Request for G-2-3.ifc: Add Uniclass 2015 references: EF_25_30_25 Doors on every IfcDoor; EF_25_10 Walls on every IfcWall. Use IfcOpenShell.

First a look at what the model holds.

```python
import ifcopenshell

model = ifcopenshell.open("G-2-3.ifc")
print(model.schema)
print("classifications:", [c.Name for c in model.by_type("IfcClassification")])
for ifc_class in ("IfcDoor", "IfcRoof", "IfcStair", "IfcWall", "IfcWindow"):
    print(ifc_class, len(model.by_type(ifc_class)))
```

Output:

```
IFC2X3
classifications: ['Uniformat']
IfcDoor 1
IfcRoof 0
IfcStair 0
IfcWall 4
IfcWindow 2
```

```python
import ifcopenshell
import ifcopenshell.api.classification

model = ifcopenshell.open("G-2-3.ifc")

# IFC2X3 requires Source and Edition and has no link from the project to the system.
system = model.create_entity("IfcClassification", Source="NBS", Edition="2015", Name="Uniclass 2015")

codes = {
    "IfcDoor": ("EF_25_30_25", "Doors"),
    "IfcWall": ("EF_25_10", "Walls"),
}
for ifc_class, (code, name) in codes.items():
    products = model.by_type(ifc_class)
    ifcopenshell.api.classification.add_reference(
        model, products=products, classification=system, identification=code, name=name
    )
    print(code, len(products))

model.write("G-2-3_updated.ifc")
```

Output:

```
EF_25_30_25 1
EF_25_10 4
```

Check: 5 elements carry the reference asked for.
